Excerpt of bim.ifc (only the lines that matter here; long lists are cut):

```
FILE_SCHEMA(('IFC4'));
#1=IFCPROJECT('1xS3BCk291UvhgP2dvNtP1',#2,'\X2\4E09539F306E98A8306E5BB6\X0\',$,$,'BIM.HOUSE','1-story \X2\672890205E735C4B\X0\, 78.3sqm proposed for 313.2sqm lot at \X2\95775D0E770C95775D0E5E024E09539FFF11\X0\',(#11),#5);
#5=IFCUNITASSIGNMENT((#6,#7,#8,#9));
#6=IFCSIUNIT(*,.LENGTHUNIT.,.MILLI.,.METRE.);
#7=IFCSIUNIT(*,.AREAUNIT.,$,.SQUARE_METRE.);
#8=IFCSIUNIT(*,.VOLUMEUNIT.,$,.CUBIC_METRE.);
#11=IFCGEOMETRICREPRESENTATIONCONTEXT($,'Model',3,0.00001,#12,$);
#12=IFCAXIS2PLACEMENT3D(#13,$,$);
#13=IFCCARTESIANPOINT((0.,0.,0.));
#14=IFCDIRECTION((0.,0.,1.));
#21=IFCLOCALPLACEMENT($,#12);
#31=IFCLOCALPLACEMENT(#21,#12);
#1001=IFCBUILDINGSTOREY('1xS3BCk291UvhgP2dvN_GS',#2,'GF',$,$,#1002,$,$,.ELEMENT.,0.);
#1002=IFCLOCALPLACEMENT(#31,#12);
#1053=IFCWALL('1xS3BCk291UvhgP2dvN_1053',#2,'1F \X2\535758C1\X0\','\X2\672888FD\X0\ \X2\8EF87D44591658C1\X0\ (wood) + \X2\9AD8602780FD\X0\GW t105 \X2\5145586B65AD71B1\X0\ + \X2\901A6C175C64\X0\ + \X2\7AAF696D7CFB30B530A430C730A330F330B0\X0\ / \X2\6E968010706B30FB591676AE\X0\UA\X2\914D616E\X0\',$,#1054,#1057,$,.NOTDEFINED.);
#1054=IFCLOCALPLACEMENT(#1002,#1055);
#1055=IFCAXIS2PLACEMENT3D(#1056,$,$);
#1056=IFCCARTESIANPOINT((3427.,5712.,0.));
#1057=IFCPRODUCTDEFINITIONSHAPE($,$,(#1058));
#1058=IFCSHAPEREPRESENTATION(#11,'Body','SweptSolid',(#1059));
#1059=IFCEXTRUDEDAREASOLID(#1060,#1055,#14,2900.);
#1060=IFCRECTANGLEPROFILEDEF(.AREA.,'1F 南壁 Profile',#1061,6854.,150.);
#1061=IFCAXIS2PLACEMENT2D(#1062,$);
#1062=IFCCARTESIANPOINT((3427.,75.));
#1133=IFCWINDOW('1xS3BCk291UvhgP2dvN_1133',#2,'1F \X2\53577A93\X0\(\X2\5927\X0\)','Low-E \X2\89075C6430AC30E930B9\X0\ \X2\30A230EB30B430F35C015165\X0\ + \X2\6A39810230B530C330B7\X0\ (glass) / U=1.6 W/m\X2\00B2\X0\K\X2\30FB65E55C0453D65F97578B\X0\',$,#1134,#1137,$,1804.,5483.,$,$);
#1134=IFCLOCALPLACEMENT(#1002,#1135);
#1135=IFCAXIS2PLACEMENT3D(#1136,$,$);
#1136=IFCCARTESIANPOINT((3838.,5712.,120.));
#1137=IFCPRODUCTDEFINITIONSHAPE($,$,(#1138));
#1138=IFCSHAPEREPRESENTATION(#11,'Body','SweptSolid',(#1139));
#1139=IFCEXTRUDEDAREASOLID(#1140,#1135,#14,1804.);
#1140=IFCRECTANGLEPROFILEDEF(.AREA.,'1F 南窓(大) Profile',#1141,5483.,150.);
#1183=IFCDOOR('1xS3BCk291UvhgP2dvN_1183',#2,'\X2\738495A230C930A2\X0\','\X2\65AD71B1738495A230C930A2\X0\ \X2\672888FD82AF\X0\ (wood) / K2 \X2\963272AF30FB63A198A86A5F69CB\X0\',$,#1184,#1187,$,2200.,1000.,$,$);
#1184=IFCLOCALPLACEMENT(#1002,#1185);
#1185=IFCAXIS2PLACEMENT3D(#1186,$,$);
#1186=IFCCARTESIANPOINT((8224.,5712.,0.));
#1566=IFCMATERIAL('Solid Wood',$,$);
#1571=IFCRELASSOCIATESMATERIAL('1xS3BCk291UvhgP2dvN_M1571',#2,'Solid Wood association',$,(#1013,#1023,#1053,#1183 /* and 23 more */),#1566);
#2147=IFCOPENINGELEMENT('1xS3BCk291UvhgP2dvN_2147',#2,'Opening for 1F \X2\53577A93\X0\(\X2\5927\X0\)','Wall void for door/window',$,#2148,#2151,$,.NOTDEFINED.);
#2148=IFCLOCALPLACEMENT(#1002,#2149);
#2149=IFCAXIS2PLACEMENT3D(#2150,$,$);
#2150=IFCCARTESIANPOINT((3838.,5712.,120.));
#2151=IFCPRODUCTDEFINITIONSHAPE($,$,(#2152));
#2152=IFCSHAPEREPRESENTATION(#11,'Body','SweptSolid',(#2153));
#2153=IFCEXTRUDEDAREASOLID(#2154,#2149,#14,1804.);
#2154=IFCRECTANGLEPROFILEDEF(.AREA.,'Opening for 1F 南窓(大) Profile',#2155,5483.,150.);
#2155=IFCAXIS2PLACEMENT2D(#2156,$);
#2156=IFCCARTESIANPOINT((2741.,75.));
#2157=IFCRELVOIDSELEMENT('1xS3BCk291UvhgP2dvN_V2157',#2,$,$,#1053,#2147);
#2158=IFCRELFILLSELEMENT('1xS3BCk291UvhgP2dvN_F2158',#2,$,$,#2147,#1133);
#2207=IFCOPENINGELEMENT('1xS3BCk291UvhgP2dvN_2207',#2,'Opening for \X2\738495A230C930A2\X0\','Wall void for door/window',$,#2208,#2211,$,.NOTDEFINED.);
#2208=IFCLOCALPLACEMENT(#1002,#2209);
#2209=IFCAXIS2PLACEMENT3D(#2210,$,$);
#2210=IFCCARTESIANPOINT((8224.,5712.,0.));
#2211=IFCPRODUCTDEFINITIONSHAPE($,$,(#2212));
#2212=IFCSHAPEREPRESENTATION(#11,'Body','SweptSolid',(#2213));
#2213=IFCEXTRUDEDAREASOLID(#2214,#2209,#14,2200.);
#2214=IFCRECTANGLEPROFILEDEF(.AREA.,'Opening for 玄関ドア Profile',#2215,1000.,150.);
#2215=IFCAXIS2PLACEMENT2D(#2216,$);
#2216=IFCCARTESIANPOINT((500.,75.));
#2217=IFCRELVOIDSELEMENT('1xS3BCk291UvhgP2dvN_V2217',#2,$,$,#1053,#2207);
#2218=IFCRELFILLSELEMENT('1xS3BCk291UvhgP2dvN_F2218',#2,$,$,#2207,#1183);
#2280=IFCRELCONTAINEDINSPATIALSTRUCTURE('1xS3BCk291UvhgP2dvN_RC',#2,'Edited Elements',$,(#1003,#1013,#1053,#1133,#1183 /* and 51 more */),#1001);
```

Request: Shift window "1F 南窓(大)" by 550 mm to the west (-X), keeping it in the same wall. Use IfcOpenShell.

```python
import ifcopenshell
import ifcopenshell.api.geometry
import ifcopenshell.util.placement
import ifcopenshell.util.unit

model = ifcopenshell.open("bim.ifc")
unit_scale = ifcopenshell.util.unit.calculate_unit_scale(model)

window = model.by_guid("1xS3BCk291UvhgP2dvN_1133")
opening = window.FillsVoids[0].RelatingOpeningElement
wall = opening.VoidsElements[0].RelatingBuildingElement

wall_matrix = ifcopenshell.util.placement.get_local_placement(wall.ObjectPlacement)
shift = wall_matrix[:3, 0] * -0.55 / unit_scale
before = ifcopenshell.util.placement.get_local_placement(window.ObjectPlacement)[:3, 3].copy()

# The window is not placed relative to its opening, so move both.
for product in (opening, window):
    matrix = ifcopenshell.util.placement.get_local_placement(product.ObjectPlacement)
    matrix[:3, 3] += shift
    ifcopenshell.api.geometry.edit_object_placement(model, product=product, matrix=matrix, is_si=False)

after = ifcopenshell.util.placement.get_local_placement(window.ObjectPlacement)[:3, 3]
print("window moved by", (after - before).round(3) + 0.0)

model.write("bim_edited.ifc")
```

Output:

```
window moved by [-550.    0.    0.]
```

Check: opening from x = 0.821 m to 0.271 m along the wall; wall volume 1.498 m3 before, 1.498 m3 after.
